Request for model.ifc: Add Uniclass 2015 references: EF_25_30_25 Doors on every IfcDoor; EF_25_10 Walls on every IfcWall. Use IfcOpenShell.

First a look at what the model holds.

```python
import ifcopenshell

model = ifcopenshell.open("model.ifc")
print(model.schema)
print("classifications:", [c.Name for c in model.by_type("IfcClassification")])
for ifc_class in ("IfcDoor", "IfcRoof", "IfcStair", "IfcWall", "IfcWindow"):
    print(ifc_class, len(model.by_type(ifc_class)))
```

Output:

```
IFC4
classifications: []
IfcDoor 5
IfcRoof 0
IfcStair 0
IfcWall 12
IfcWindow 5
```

```python
import ifcopenshell
import ifcopenshell.api.classification

model = ifcopenshell.open("model.ifc")

system = ifcopenshell.api.classification.add_classification(model, classification="Uniclass 2015")

codes = {
    "IfcDoor": ("EF_25_30_25", "Doors"),
    "IfcWall": ("EF_25_10", "Walls"),
}
for ifc_class, (code, name) in codes.items():
    products = model.by_type(ifc_class)
    ifcopenshell.api.classification.add_reference(
        model, products=products, classification=system, identification=code, name=name
    )
    print(code, len(products))

model.write("model_edited.ifc")
```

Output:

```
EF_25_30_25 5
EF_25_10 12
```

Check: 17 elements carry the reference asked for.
